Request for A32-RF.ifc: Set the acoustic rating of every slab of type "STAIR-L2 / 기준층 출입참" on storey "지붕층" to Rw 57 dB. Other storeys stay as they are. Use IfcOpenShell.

First a look at what the model holds.

```python
import ifcopenshell
import ifcopenshell.util.element

model = ifcopenshell.open("A32-RF.ifc")
print(model.schema)
storey = next(s for s in model.by_type("IfcBuildingStorey") if s.Name == "지붕층")
slabs = [e for e in ifcopenshell.util.element.get_decomposition(storey) if e.is_a("IfcSlab")]
seen = {}
for e in slabs:
    element_type = ifcopenshell.util.element.get_type(e)
    key = (element_type.Name if element_type != e and element_type else None, ifcopenshell.util.element.get_pset(e, "Pset_SlabCommon", "AcousticRating"))
    seen[key] = seen.get(key, 0) + 1
for (name, value), count in sorted(seen.items(), key=str):
    print(count, "x", name, "|", value)
```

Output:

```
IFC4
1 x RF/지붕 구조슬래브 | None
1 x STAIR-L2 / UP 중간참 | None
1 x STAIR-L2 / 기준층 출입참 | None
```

```python
import ifcopenshell
import ifcopenshell.api.pset
import ifcopenshell.util.element

model = ifcopenshell.open("A32-RF.ifc")

storey = next(s for s in model.by_type("IfcBuildingStorey") if s.Name == "지붕층")
slabs = [e for e in ifcopenshell.util.element.get_decomposition(storey) if e.is_a("IfcSlab")]

count = 0
for e in slabs:
    element_type = ifcopenshell.util.element.get_type(e)
    if element_type in (None, e) or element_type.Name != "STAIR-L2 / 기준층 출입참":
        continue
    # add_pset returns the element's existing set when there is one.
    pset = ifcopenshell.api.pset.add_pset(model, product=e, name="Pset_SlabCommon")
    ifcopenshell.api.pset.edit_pset(model, pset=pset, properties={"AcousticRating": "Rw 57 dB"})
    count += 1

print(count, "slabs updated")

model.write("A32-RF_edited.ifc")
```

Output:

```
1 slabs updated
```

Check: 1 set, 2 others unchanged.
